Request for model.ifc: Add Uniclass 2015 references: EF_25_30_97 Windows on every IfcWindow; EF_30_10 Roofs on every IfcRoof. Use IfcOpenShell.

First a look at what the model holds.

```python
import ifcopenshell

model = ifcopenshell.open("model.ifc")
print(model.schema)
print("classifications:", [c.Name for c in model.by_type("IfcClassification")])
for ifc_class in ("IfcDoor", "IfcRoof", "IfcStair", "IfcWall", "IfcWindow"):
    print(ifc_class, len(model.by_type(ifc_class)))
```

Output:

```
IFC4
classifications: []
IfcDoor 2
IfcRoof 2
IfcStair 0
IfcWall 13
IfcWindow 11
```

```python
import ifcopenshell
import ifcopenshell.api.classification

model = ifcopenshell.open("model.ifc")

system = ifcopenshell.api.classification.add_classification(model, classification="Uniclass 2015")

codes = {
    "IfcWindow": ("EF_25_30_97", "Windows"),
    "IfcRoof": ("EF_30_10", "Roofs"),
}
for ifc_class, (code, name) in codes.items():
    products = model.by_type(ifc_class)
    ifcopenshell.api.classification.add_reference(
        model, products=products, classification=system, identification=code, name=name
    )
    print(code, len(products))

model.write("model-out.ifc")
```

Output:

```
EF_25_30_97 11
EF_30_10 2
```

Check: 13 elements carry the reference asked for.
